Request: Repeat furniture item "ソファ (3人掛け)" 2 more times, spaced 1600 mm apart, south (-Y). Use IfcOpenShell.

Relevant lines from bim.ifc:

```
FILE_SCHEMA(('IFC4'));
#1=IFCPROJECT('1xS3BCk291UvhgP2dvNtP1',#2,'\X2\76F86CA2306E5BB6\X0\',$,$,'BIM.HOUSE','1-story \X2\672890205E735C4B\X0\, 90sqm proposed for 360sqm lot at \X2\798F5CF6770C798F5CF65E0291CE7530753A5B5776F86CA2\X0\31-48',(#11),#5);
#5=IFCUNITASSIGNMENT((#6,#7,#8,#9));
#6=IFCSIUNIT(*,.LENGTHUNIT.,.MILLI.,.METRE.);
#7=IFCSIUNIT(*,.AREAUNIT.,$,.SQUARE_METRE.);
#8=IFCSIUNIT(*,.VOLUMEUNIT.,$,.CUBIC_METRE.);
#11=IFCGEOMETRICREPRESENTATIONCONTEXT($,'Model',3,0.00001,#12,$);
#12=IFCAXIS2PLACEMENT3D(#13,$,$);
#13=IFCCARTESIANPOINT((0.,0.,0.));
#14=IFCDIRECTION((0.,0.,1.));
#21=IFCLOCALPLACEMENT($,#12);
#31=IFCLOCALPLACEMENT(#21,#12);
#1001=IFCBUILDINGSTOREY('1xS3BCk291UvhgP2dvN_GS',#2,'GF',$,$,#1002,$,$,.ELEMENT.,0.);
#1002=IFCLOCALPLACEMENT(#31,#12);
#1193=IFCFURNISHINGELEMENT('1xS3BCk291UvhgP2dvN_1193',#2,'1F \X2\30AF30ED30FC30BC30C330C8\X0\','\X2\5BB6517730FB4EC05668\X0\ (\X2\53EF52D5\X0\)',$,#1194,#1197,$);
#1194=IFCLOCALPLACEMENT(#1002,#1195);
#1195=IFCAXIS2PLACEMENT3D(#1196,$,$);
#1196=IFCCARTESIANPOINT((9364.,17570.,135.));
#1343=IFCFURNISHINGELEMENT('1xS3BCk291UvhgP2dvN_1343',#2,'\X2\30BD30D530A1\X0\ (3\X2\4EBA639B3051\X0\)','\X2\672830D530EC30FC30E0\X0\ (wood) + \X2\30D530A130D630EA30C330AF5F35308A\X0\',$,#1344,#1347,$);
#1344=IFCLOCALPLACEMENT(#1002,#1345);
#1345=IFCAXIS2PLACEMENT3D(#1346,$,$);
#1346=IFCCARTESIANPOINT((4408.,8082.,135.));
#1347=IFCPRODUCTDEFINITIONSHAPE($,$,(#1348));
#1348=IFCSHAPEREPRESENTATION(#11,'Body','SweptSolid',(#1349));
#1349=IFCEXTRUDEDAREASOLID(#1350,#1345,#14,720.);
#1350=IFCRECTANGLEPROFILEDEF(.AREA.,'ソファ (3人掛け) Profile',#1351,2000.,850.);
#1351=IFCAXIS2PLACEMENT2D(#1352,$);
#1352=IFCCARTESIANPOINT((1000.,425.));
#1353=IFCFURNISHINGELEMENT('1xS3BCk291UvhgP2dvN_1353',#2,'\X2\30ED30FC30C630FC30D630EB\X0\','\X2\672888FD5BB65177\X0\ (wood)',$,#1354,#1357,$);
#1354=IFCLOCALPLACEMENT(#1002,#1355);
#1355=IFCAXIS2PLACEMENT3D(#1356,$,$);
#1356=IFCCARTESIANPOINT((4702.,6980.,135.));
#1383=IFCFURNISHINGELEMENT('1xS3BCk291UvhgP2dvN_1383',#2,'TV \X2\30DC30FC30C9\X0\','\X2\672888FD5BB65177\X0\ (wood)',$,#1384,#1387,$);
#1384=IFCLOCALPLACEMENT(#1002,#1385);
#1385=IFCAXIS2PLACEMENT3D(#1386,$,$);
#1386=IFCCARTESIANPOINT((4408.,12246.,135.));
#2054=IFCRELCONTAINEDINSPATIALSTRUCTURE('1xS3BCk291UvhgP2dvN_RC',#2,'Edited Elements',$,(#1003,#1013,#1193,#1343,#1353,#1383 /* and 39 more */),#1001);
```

```python
import numpy as np
import ifcopenshell
import ifcopenshell.api.geometry
import ifcopenshell.api.root
import ifcopenshell.util.element
import ifcopenshell.util.placement

model = ifcopenshell.open("bim.ifc")


def reuse_history(source, copy):
    """copy_class also copies each property set's owner history, people and application; keep the originals."""
    for rel in copy.IsDefinedBy:
        if rel.is_a("IfcRelDefinesByProperties") and (history := rel.RelatingPropertyDefinition.OwnerHistory):
            rel.RelatingPropertyDefinition.OwnerHistory = source.OwnerHistory
            ifcopenshell.util.element.remove_deep2(model, history)


source = model.by_guid("1xS3BCk291UvhgP2dvN_1343")
base = ifcopenshell.util.placement.get_local_placement(source.ObjectPlacement)
step = np.array([0.0, -1.0, 0.0]) * 1600.0

for i in range(1, 3):
    copy = ifcopenshell.api.root.copy_class(model, product=source)
    copy.Representation = ifcopenshell.util.element.copy_deep(
        model, source.Representation, exclude=["IfcGeometricRepresentationContext", "IfcRepresentationMap"]
    )
    reuse_history(source, copy)
    matrix = base.copy()
    matrix[:3, 3] += i * step
    print("added at", matrix[:3, 3].round(3) + 0.0)
    ifcopenshell.api.geometry.edit_object_placement(model, product=copy, matrix=matrix, is_si=False)

model.write("bim_rev.ifc")
```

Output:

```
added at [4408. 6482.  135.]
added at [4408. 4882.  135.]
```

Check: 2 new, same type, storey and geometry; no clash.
